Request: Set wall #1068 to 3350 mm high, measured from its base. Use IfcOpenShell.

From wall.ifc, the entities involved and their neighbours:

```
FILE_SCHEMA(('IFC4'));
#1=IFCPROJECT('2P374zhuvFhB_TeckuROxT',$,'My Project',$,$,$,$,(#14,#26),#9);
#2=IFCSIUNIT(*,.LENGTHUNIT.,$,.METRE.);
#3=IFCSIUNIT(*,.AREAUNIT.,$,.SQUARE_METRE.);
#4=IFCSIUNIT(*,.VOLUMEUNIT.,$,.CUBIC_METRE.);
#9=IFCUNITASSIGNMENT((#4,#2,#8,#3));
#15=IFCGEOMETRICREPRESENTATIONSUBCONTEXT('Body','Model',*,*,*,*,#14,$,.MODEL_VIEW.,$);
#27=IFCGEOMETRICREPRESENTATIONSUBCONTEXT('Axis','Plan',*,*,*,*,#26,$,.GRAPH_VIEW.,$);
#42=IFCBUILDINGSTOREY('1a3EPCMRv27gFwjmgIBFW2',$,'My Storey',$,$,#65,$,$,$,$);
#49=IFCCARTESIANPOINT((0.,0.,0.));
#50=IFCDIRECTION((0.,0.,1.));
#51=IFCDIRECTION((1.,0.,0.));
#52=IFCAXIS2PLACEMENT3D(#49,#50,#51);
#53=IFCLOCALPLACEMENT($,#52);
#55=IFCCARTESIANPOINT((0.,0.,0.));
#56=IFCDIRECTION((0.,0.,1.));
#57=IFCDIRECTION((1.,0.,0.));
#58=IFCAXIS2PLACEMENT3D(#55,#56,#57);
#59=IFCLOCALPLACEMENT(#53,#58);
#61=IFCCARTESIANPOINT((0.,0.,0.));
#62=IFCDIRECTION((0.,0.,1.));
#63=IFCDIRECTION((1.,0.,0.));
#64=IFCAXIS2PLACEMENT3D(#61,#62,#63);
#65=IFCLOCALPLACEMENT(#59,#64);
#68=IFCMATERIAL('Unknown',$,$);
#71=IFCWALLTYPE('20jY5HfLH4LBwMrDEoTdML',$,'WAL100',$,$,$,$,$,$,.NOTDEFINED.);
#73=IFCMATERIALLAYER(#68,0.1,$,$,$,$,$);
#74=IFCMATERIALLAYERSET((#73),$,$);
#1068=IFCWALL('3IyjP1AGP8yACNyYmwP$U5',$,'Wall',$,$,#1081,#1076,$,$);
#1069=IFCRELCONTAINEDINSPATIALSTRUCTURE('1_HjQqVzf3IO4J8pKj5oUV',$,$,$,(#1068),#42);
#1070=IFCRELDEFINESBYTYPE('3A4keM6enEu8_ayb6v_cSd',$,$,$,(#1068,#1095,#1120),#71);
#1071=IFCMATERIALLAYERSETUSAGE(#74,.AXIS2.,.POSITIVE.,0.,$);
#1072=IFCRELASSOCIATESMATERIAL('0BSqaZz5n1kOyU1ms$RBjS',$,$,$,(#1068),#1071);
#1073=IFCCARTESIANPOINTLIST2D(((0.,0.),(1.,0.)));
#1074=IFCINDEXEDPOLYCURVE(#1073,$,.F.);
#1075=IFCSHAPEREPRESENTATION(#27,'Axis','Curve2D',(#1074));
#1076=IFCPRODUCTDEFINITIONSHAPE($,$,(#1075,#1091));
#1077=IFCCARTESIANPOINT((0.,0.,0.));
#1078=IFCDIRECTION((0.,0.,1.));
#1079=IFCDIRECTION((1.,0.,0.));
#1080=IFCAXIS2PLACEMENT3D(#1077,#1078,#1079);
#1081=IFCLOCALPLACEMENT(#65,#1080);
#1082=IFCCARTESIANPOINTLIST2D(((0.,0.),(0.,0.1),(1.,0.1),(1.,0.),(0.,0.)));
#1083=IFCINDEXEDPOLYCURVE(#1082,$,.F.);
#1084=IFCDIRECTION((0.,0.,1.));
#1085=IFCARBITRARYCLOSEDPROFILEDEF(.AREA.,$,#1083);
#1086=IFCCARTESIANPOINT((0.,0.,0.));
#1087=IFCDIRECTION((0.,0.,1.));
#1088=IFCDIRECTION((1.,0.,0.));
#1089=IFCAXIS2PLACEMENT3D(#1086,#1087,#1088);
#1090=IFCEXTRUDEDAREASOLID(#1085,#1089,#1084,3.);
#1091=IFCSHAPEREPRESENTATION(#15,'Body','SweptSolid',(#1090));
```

```python
import ifcopenshell
import ifcopenshell.geom
import ifcopenshell.util.representation
import ifcopenshell.util.shape
import ifcopenshell.util.unit

model = ifcopenshell.open("wall.ifc")
unit_scale = ifcopenshell.util.unit.calculate_unit_scale(model)
settings = ifcopenshell.geom.settings()


def volume(element):
    """Net volume in cubic metres, openings subtracted."""
    shape = ifcopenshell.geom.create_shape(settings, element)
    return ifcopenshell.util.shape.get_volume(shape.geometry)


wall = model.by_guid("3IyjP1AGP8yACNyYmwP$U5")
before = volume(wall)

body = ifcopenshell.util.representation.get_representation(wall, "Model", "Body")
solid = body.Items[0]
old_height = solid.Depth
solid.Depth = 3.35 / unit_scale
after = volume(wall)

print(f"height {old_height:g} -> {solid.Depth:g}, volume {before:.3f} -> {after:.3f} m3")

model.write("wall_v2.ifc")
```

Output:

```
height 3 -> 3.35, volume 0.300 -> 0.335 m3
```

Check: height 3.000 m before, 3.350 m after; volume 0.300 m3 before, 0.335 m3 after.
